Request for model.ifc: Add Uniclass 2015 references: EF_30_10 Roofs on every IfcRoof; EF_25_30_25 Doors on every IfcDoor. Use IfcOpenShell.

First a look at what the model holds.

```python
import ifcopenshell

model = ifcopenshell.open("model.ifc")
print(model.schema)
print("classifications:", [c.Name for c in model.by_type("IfcClassification")])
for ifc_class in ("IfcDoor", "IfcRoof", "IfcStair", "IfcWall", "IfcWindow"):
    print(ifc_class, len(model.by_type(ifc_class)))
```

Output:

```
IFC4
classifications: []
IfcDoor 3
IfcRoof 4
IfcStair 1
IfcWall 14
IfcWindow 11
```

```python
import ifcopenshell
import ifcopenshell.api.classification

model = ifcopenshell.open("model.ifc")

system = ifcopenshell.api.classification.add_classification(model, classification="Uniclass 2015")

codes = {
    "IfcRoof": ("EF_30_10", "Roofs"),
    "IfcDoor": ("EF_25_30_25", "Doors"),
}
for ifc_class, (code, name) in codes.items():
    products = model.by_type(ifc_class)
    ifcopenshell.api.classification.add_reference(
        model, products=products, classification=system, identification=code, name=name
    )
    print(code, len(products))

model.write("model_rev.ifc")
```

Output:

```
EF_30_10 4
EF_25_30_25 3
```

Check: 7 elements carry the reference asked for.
